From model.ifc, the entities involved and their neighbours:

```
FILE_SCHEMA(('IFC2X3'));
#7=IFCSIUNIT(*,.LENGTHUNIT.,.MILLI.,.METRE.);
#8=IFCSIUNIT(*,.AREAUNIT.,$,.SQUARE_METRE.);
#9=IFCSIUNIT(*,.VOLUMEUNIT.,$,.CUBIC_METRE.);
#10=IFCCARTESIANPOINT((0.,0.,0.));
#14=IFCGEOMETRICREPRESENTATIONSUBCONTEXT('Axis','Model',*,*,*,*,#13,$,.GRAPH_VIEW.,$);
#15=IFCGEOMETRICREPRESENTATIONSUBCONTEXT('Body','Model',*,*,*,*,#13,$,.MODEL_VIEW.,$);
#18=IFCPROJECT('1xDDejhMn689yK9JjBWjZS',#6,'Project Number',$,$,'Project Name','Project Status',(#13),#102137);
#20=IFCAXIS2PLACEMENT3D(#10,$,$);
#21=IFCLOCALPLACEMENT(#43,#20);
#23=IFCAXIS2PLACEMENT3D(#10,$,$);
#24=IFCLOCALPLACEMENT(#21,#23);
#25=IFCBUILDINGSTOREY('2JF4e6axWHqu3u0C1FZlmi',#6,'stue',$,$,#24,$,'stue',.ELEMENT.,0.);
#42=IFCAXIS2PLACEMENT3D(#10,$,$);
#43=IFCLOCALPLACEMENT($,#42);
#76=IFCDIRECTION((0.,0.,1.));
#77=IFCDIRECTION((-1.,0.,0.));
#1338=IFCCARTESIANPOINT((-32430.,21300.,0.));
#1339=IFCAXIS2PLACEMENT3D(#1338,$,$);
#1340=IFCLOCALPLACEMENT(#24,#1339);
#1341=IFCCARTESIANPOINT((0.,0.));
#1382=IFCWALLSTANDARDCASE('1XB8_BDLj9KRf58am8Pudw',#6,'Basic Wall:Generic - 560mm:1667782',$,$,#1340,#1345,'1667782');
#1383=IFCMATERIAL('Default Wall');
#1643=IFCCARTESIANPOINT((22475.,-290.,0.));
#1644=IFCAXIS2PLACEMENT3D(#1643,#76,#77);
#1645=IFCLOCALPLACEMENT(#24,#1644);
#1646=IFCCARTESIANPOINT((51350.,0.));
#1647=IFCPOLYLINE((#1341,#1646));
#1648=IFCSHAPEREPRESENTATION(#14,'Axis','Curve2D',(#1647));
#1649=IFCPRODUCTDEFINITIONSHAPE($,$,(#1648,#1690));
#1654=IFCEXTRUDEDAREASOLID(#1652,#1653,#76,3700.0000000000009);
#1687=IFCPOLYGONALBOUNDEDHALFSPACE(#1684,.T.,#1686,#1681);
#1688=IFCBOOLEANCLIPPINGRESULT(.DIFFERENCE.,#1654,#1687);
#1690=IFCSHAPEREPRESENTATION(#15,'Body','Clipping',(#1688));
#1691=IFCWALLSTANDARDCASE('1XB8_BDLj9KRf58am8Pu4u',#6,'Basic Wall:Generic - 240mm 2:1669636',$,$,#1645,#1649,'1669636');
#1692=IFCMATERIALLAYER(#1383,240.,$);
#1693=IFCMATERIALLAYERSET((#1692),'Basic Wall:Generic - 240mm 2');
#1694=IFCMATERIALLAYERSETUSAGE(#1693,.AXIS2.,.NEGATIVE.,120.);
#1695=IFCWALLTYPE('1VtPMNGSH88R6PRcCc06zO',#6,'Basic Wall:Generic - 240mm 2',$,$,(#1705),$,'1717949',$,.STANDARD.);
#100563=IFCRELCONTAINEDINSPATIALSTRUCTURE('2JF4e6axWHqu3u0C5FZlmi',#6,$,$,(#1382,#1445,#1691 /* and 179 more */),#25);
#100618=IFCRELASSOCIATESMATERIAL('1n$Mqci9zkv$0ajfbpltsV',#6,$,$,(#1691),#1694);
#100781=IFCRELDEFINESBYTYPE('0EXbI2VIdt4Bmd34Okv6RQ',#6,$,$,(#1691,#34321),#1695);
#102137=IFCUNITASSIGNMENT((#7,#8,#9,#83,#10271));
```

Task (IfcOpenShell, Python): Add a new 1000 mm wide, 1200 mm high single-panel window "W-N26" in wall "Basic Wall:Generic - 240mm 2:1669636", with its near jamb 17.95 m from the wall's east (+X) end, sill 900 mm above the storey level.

```python
import numpy as np
import ifcopenshell
import ifcopenshell.api.feature
import ifcopenshell.api.geometry
import ifcopenshell.api.root
import ifcopenshell.api.spatial
import ifcopenshell.api.type
import ifcopenshell.geom
import ifcopenshell.util.element
import ifcopenshell.util.placement
import ifcopenshell.util.representation
import ifcopenshell.util.shape
import ifcopenshell.util.unit

model = ifcopenshell.open("model.ifc")
unit_scale = ifcopenshell.util.unit.calculate_unit_scale(model)
settings = ifcopenshell.geom.settings()


def volume(element):
    """Net volume in cubic metres, openings subtracted."""
    shape = ifcopenshell.geom.create_shape(settings, element)
    return ifcopenshell.util.shape.get_volume(shape.geometry)


wall = model.by_guid("1XB8_BDLj9KRf58am8Pu4u")
storey = ifcopenshell.util.element.get_container(wall, ifc_class="IfcBuildingStorey")
context = ifcopenshell.util.representation.get_context(model, "Model", "Body", "MODEL_VIEW")
before = volume(wall)

width, height, from_end, sill = 1, 1.2, 17.95, 0.9  # metres

# The wall runs along its own X axis, and the end named is its -X end.
wall_shape = ifcopenshell.geom.create_shape(settings, wall)
x, y, z = ifcopenshell.util.shape.get_vertices(wall_shape.geometry).T
start = x.min() + from_end
face, thickness = float(y.min()), float(y.max() - y.min())
wall_matrix = ifcopenshell.util.placement.get_local_placement(wall.ObjectPlacement)
level = ifcopenshell.util.placement.get_local_placement(storey.ObjectPlacement)[2, 3]


def in_wall(x, y):
    """Placement at x, y metres in the wall's axes, at sill height."""
    matrix = wall_matrix.copy()
    matrix[:, 3] = wall_matrix @ np.array([x / unit_scale, y / unit_scale, 0.0, 1.0])
    matrix[2, 3] = level + sill / unit_scale
    return matrix


# Opening: a box that overshoots both wall faces by 50 mm.
opening = ifcopenshell.api.root.create_entity(model, ifc_class="IfcOpeningElement")
box = ifcopenshell.api.geometry.add_wall_representation(
    model, context=context, length=width, height=height, thickness=thickness + 0.1
)
ifcopenshell.api.geometry.assign_representation(model, product=opening, representation=box)
ifcopenshell.api.geometry.edit_object_placement(model, product=opening, matrix=in_wall(start, face - 0.05), is_si=False)
ifcopenshell.api.feature.add_feature(model, feature=opening, element=wall)

window = ifcopenshell.api.root.create_entity(model, ifc_class="IfcWindow", name="W-N26")
window.OverallWidth, window.OverallHeight = width / unit_scale, height / unit_scale
body = ifcopenshell.api.geometry.add_window_representation(
    model,
    context=context,
    overall_width=window.OverallWidth,
    overall_height=window.OverallHeight,
    partition_type="SINGLE_PANEL",
)
ifcopenshell.api.geometry.assign_representation(model, product=window, representation=body)
ifcopenshell.api.spatial.assign_container(model, products=[window], relating_structure=storey)
fills = ifcopenshell.api.feature.add_filling(model, opening=opening, element=window)
fills.OwnerHistory = window.OwnerHistory  # required in IFC2X3

# IFC2X3 keeps the operation on the window style.
style = ifcopenshell.api.root.create_entity(model, ifc_class="IfcWindowStyle", name="W-N26")
style.OperationType, style.ConstructionType = "SINGLE_PANEL", "NOTDEFINED"
style.ParameterTakesPrecedence = style.Sizeable = False
ifcopenshell.api.type.assign_type(model, related_objects=[window], relating_type=style)

# Centre the window in the wall's thickness.
ifcopenshell.api.geometry.edit_object_placement(model, product=window, matrix=in_wall(start, face), is_si=False)
window_shape = ifcopenshell.geom.create_shape(settings, window)
depth = ifcopenshell.util.shape.get_vertices(window_shape.geometry)[:, 1]
offset = face + thickness / 2 - (depth.min() + depth.max()) / 2
ifcopenshell.api.geometry.edit_object_placement(model, product=window, matrix=in_wall(start, offset), is_si=False)

after = volume(wall)

print(f"wall volume {before:.3f} -> {after:.3f} m3")

model.write("model_edited.ifc")
```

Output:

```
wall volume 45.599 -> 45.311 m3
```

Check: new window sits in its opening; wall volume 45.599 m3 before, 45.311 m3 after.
